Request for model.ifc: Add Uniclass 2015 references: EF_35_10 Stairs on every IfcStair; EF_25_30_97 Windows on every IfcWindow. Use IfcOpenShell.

First a look at what the model holds.

```python
import ifcopenshell

model = ifcopenshell.open("model.ifc")
print(model.schema)
print("classifications:", [c.Name for c in model.by_type("IfcClassification")])
for ifc_class in ("IfcDoor", "IfcRoof", "IfcStair", "IfcWall", "IfcWindow"):
    print(ifc_class, len(model.by_type(ifc_class)))
```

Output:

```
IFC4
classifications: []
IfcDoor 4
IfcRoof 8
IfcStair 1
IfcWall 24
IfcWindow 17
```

```python
import ifcopenshell
import ifcopenshell.api.classification

model = ifcopenshell.open("model.ifc")

system = ifcopenshell.api.classification.add_classification(model, classification="Uniclass 2015")

codes = {
    "IfcStair": ("EF_35_10", "Stairs"),
    "IfcWindow": ("EF_25_30_97", "Windows"),
}
for ifc_class, (code, name) in codes.items():
    products = model.by_type(ifc_class)
    ifcopenshell.api.classification.add_reference(
        model, products=products, classification=system, identification=code, name=name
    )
    print(code, len(products))

model.write("model_v2.ifc")
```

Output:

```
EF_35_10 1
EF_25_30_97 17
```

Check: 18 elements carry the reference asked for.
